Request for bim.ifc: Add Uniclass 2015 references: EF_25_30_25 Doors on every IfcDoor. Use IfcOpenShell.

First a look at what the model holds.

```python
import ifcopenshell

model = ifcopenshell.open("bim.ifc")
print(model.schema)
print("classifications:", [c.Name for c in model.by_type("IfcClassification")])
for ifc_class in ("IfcDoor", "IfcRoof", "IfcStair", "IfcWall", "IfcWindow"):
    print(ifc_class, len(model.by_type(ifc_class)))
```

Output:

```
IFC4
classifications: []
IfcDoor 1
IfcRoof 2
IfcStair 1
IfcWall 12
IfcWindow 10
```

```python
import ifcopenshell
import ifcopenshell.api.classification

model = ifcopenshell.open("bim.ifc")

system = ifcopenshell.api.classification.add_classification(model, classification="Uniclass 2015")

codes = {
    "IfcDoor": ("EF_25_30_25", "Doors"),
}
for ifc_class, (code, name) in codes.items():
    products = model.by_type(ifc_class)
    ifcopenshell.api.classification.add_reference(
        model, products=products, classification=system, identification=code, name=name
    )
    print(code, len(products))

model.write("bim_rev.ifc")
```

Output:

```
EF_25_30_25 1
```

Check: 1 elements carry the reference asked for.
